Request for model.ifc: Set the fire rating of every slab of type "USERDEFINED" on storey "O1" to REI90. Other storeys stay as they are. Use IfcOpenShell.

First a look at what the model holds.

```python
import ifcopenshell
import ifcopenshell.util.element

model = ifcopenshell.open("model.ifc")
print(model.schema)
storey = next(s for s in model.by_type("IfcBuildingStorey") if s.Name == "O1")
slabs = [e for e in ifcopenshell.util.element.get_decomposition(storey) if e.is_a("IfcSlab")]
seen = {}
for e in slabs:
    element_type = ifcopenshell.util.element.get_type(e)
    key = (element_type.Name if element_type != e and element_type else None, ifcopenshell.util.element.get_pset(e, "Pset_SlabCommon", "FireRating"))
    seen[key] = seen.get(key, 0) + 1
for (name, value), count in sorted(seen.items(), key=str):
    print(count, "x", name, "|", value)
```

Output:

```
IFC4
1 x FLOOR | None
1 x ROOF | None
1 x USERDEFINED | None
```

```python
import ifcopenshell
import ifcopenshell.api.pset
import ifcopenshell.util.element

model = ifcopenshell.open("model.ifc")

storey = next(s for s in model.by_type("IfcBuildingStorey") if s.Name == "O1")
slabs = [e for e in ifcopenshell.util.element.get_decomposition(storey) if e.is_a("IfcSlab")]

count = 0
for e in slabs:
    element_type = ifcopenshell.util.element.get_type(e)
    if element_type in (None, e) or element_type.Name != "USERDEFINED":
        continue
    # add_pset returns the element's existing set when there is one.
    pset = ifcopenshell.api.pset.add_pset(model, product=e, name="Pset_SlabCommon")
    ifcopenshell.api.pset.edit_pset(model, pset=pset, properties={"FireRating": "REI90"})
    count += 1

print(count, "slabs updated")

model.write("model_v2.ifc")
```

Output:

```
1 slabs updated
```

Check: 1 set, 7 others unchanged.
